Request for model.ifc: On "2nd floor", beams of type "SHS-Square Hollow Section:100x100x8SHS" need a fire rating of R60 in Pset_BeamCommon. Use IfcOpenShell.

First a look at what the model holds.

```python
import ifcopenshell
import ifcopenshell.util.element

model = ifcopenshell.open("model.ifc")
print(model.schema)
storey = next(s for s in model.by_type("IfcBuildingStorey") if s.Name == "2nd floor")
beams = [e for e in ifcopenshell.util.element.get_decomposition(storey) if e.is_a("IfcBeam")]
seen = {}
for e in beams:
    element_type = ifcopenshell.util.element.get_type(e)
    key = (element_type.Name if element_type != e and element_type else None, ifcopenshell.util.element.get_pset(e, "Pset_BeamCommon", "FireRating"))
    seen[key] = seen.get(key, 0) + 1
for (name, value), count in sorted(seen.items(), key=str):
    print(count, "x", name, "|", value)
```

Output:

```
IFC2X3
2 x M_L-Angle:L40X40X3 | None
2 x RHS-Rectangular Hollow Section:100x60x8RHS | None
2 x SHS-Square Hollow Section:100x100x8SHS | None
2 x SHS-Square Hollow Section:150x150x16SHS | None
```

```python
import ifcopenshell
import ifcopenshell.api.pset
import ifcopenshell.util.element

model = ifcopenshell.open("model.ifc")

storey = next(s for s in model.by_type("IfcBuildingStorey") if s.Name == "2nd floor")
beams = [e for e in ifcopenshell.util.element.get_decomposition(storey) if e.is_a("IfcBeam")]

count = 0
for e in beams:
    element_type = ifcopenshell.util.element.get_type(e)
    if element_type in (None, e) or element_type.Name != "SHS-Square Hollow Section:100x100x8SHS":
        continue
    # add_pset returns the element's existing set when there is one.
    pset = ifcopenshell.api.pset.add_pset(model, product=e, name="Pset_BeamCommon")
    ifcopenshell.api.pset.edit_pset(model, pset=pset, properties={"FireRating": "R60"})
    count += 1

print(count, "beams updated")

model.write("model-out.ifc")
```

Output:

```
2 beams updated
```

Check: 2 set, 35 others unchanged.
